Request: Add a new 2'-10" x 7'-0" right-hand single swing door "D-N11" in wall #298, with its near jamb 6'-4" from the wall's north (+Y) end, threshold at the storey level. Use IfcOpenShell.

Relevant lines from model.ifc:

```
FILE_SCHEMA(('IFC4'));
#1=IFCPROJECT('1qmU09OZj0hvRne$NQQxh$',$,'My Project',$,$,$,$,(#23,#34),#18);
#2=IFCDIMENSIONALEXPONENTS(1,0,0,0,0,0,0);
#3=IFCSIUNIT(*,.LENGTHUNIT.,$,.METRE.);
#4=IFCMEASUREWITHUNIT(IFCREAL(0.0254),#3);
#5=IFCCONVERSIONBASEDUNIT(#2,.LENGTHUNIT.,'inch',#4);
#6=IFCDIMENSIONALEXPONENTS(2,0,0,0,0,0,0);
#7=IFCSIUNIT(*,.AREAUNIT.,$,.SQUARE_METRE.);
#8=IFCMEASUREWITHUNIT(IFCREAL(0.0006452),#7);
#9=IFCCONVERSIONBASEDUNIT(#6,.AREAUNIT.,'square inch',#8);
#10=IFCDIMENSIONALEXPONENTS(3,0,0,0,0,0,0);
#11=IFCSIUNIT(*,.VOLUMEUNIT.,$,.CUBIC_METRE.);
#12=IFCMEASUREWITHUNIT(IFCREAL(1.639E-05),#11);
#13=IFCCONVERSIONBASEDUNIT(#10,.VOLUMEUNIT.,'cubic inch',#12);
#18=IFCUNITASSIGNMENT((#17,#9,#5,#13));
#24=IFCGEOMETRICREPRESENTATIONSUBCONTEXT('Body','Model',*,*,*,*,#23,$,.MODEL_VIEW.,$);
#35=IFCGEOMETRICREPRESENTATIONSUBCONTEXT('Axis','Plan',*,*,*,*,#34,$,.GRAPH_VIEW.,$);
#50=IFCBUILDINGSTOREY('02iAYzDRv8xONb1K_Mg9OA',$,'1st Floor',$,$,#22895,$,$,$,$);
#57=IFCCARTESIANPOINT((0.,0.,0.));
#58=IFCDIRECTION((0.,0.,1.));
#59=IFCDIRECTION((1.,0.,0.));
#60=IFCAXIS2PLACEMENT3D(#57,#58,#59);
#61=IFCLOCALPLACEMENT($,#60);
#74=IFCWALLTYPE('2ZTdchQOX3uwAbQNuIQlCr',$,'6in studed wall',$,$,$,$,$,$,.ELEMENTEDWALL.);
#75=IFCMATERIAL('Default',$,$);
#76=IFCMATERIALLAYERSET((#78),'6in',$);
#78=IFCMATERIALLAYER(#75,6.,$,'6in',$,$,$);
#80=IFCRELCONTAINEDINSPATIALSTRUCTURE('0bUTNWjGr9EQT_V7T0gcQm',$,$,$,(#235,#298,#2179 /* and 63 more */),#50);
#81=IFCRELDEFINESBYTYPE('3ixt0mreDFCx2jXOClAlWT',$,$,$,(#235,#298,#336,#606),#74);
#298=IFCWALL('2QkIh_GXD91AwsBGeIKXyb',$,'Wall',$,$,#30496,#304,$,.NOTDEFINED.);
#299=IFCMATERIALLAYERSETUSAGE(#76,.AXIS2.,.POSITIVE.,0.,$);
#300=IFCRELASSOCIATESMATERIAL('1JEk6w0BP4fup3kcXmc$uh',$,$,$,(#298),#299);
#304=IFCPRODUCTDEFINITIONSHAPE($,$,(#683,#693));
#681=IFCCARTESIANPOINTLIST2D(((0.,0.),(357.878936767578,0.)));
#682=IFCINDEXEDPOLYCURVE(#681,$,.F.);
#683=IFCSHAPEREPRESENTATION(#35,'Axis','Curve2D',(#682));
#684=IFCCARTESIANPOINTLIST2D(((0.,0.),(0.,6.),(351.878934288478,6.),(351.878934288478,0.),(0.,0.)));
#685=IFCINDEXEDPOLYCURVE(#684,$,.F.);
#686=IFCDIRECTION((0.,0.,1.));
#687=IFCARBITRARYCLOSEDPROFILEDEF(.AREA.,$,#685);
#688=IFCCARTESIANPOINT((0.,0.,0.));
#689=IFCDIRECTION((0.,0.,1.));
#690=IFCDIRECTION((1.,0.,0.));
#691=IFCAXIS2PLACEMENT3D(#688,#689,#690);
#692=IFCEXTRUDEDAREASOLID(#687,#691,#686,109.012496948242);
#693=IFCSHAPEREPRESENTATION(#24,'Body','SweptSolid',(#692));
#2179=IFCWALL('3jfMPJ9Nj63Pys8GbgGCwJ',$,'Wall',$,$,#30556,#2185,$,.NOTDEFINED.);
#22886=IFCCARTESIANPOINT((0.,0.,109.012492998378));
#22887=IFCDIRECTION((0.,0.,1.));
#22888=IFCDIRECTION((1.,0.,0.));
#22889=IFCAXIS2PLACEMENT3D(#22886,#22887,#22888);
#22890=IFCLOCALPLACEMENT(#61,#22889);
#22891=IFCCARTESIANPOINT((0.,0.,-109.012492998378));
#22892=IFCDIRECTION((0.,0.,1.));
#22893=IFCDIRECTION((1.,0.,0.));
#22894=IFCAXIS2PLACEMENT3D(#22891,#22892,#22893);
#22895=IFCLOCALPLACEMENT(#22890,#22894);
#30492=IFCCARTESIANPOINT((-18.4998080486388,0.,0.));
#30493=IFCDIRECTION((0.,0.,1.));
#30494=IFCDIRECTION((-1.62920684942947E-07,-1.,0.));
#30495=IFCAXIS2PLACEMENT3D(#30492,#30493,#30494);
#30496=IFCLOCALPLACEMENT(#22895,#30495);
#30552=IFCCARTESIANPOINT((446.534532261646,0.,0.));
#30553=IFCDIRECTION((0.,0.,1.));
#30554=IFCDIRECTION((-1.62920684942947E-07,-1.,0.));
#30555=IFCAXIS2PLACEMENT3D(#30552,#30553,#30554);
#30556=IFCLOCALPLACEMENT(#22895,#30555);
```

```python
import numpy as np
import ifcopenshell
import ifcopenshell.api.feature
import ifcopenshell.api.geometry
import ifcopenshell.api.root
import ifcopenshell.api.spatial
import ifcopenshell.geom
import ifcopenshell.util.element
import ifcopenshell.util.placement
import ifcopenshell.util.representation
import ifcopenshell.util.shape
import ifcopenshell.util.unit

model = ifcopenshell.open("model.ifc")
unit_scale = ifcopenshell.util.unit.calculate_unit_scale(model)
settings = ifcopenshell.geom.settings()


def volume(element):
    """Net volume in cubic metres, openings subtracted."""
    shape = ifcopenshell.geom.create_shape(settings, element)
    return ifcopenshell.util.shape.get_volume(shape.geometry)


wall = model.by_guid("2QkIh_GXD91AwsBGeIKXyb")
storey = ifcopenshell.util.element.get_container(wall, ifc_class="IfcBuildingStorey")
context = ifcopenshell.util.representation.get_context(model, "Model", "Body", "MODEL_VIEW")
before = volume(wall)

width, height, from_end, sill = 0.8636, 2.1336, 1.9304, 0.0  # metres

# The wall runs along its own X axis, and the end named is its -X end.
wall_shape = ifcopenshell.geom.create_shape(settings, wall)
x, y, z = ifcopenshell.util.shape.get_vertices(wall_shape.geometry).T
start = x.min() + from_end
face, thickness = float(y.min()), float(y.max() - y.min())
wall_matrix = ifcopenshell.util.placement.get_local_placement(wall.ObjectPlacement)
level = ifcopenshell.util.placement.get_local_placement(storey.ObjectPlacement)[2, 3]


def in_wall(x, y):
    """Placement at x, y metres in the wall's axes, at sill height."""
    matrix = wall_matrix.copy()
    matrix[:, 3] = wall_matrix @ np.array([x / unit_scale, y / unit_scale, 0.0, 1.0])
    matrix[2, 3] = level + sill / unit_scale
    return matrix


# Opening: a box that overshoots both wall faces by 50 mm.
opening = ifcopenshell.api.root.create_entity(model, ifc_class="IfcOpeningElement", predefined_type="OPENING")
box = ifcopenshell.api.geometry.add_wall_representation(
    model, context=context, length=width, height=height, thickness=thickness + 0.1
)
ifcopenshell.api.geometry.assign_representation(model, product=opening, representation=box)
ifcopenshell.api.geometry.edit_object_placement(model, product=opening, matrix=in_wall(start, face - 0.05), is_si=False)
ifcopenshell.api.feature.add_feature(model, feature=opening, element=wall)

door = ifcopenshell.api.root.create_entity(model, ifc_class="IfcDoor", name="D-N11", predefined_type="DOOR")
door.OverallWidth, door.OverallHeight = width / unit_scale, height / unit_scale
door.OperationType = "SINGLE_SWING_RIGHT"
body = ifcopenshell.api.geometry.add_door_representation(
    model,
    context=context,
    overall_width=door.OverallWidth,
    overall_height=door.OverallHeight,
    operation_type="SINGLE_SWING_RIGHT",
    lining_properties={"LiningDepth": thickness / unit_scale, "ThresholdDepth": thickness / unit_scale},
)
ifcopenshell.api.geometry.assign_representation(model, product=door, representation=body)
ifcopenshell.api.spatial.assign_container(model, products=[door], relating_structure=storey)
ifcopenshell.api.feature.add_filling(model, opening=opening, element=door)

# The lining spans the wall, so the door starts at the wall face.
ifcopenshell.api.geometry.edit_object_placement(model, product=door, matrix=in_wall(start, face), is_si=False)

after = volume(wall)

print(f"wall volume {before:.3f} -> {after:.3f} m3")

model.write("model_v2.ifc")
```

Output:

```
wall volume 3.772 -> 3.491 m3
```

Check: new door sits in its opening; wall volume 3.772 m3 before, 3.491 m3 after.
